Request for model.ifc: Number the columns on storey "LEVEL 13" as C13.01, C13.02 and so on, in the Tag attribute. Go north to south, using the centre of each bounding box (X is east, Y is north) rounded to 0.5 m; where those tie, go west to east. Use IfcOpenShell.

First a look at what the model holds.

```python
import ifcopenshell
import ifcopenshell.util.element
import ifcopenshell.util.placement

model = ifcopenshell.open("model.ifc")
print(model.schema)
storey = next(s for s in model.by_type("IfcBuildingStorey") if s.Name == "LEVEL 13")
columns = [e for e in ifcopenshell.util.element.get_decomposition(storey) if e.is_a("IfcColumn")]
for e in sorted(columns, key=lambda e: e.id()):
    origin = ifcopenshell.util.placement.get_local_placement(e.ObjectPlacement)[:3, 3]
    print(e.id(), e.Tag, e.Name, origin.round(2) + 0.0, sep=" | ")
```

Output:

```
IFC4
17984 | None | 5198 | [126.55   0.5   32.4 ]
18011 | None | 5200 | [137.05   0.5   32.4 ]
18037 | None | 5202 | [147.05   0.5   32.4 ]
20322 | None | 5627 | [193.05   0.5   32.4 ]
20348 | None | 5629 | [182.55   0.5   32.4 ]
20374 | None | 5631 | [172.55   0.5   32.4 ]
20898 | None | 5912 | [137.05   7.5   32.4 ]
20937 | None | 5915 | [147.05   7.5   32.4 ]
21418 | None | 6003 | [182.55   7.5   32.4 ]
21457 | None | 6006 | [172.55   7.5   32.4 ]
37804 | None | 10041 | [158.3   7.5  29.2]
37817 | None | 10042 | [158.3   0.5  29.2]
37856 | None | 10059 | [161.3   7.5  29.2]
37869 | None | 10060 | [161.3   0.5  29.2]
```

```python
import ifcopenshell
import ifcopenshell.geom
import ifcopenshell.util.element
import ifcopenshell.util.shape

model = ifcopenshell.open("model.ifc")
settings = ifcopenshell.geom.settings()
settings.set("use-world-coords", True)


def centre(element):
    shape = ifcopenshell.geom.create_shape(settings, element)
    return ifcopenshell.util.shape.get_bbox_centroid(shape.geometry)


storey = next(s for s in model.by_type("IfcBuildingStorey") if s.Name == "LEVEL 13")
columns = [e for e in ifcopenshell.util.element.get_decomposition(storey) if e.is_a("IfcColumn")]

# Insertion points can sit at a corner or the storey origin, so sort by the geometry (in metres).
centres = {e: centre(e) for e in columns}
columns.sort(key=lambda e: (-round(centres[e][1] / 0.5), centres[e][0]))

for i, e in enumerate(columns, start=1):
    number = f"C13.{i:02d}"
    e.Tag = number
    print(e.id(), number)

model.write("model_rev.ifc")
```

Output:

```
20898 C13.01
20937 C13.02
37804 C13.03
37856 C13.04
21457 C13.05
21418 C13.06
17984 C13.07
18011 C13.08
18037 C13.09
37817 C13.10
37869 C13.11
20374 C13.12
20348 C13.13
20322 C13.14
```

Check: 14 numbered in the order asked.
